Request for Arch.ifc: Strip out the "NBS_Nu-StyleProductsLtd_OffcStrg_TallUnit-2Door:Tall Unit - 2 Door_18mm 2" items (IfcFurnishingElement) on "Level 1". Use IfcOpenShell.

First a look at what the model holds.

```python
import ifcopenshell
import ifcopenshell.util.element

model = ifcopenshell.open("Arch.ifc")
print(model.schema)
storey = next(s for s in model.by_type("IfcBuildingStorey") if s.Name == "Level 1")
furniture = [e for e in ifcopenshell.util.element.get_decomposition(storey) if e.is_a("IfcFurnishingElement")]
seen = {}
for e in furniture:
    element_type = ifcopenshell.util.element.get_type(e)
    name = element_type.Name if element_type not in (None, e) else None
    seen[name] = seen.get(name, 0) + 1
for name, count in sorted(seen.items(), key=str):
    print(count, "x", name)
```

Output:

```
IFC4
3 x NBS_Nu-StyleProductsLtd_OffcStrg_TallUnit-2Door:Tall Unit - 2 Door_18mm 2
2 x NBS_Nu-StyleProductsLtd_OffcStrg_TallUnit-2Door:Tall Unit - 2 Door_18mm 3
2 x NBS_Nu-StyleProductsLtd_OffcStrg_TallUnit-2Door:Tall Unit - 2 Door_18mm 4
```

```python
import ifcopenshell
import ifcopenshell.api.root
import ifcopenshell.util.element

model = ifcopenshell.open("Arch.ifc")

storey = next(s for s in model.by_type("IfcBuildingStorey") if s.Name == "Level 1")
furniture = [e for e in ifcopenshell.util.element.get_decomposition(storey) if e.is_a("IfcFurnishingElement")]
targets = [e for e in furniture if (t := ifcopenshell.util.element.get_type(e)) not in (None, e) and t.Name == "NBS_Nu-StyleProductsLtd_OffcStrg_TallUnit-2Door:Tall Unit - 2 Door_18mm 2"]

for e in targets:
    ifcopenshell.api.root.remove_product(model, product=e)
print(len(targets), "removed")

model.write("Arch-out.ifc")
```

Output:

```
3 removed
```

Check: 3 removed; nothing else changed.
